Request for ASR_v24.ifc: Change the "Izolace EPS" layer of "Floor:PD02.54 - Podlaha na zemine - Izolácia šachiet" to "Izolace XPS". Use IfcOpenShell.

First a look at what the model holds.

```python
import ifcopenshell
import ifcopenshell.util.element

model = ifcopenshell.open("ASR_v24.ifc")
print(model.schema)
for layer_set in model.by_type("IfcMaterialLayerSet"):
    if layer_set.LayerSetName == "Floor:PD02.54 - Podlaha na zemine - Izolácia šachiet":
        for layer in layer_set.MaterialLayers:
            print(layer.id(), layer.Material and layer.Material.Name, layer.LayerThickness, sep=" | ")
        print(len(ifcopenshell.util.element.get_elements_by_material(model, layer_set)), "elements and types use it")
print(sorted(m.Name for m in model.by_type("IfcMaterial") if m.Name)[:60])
```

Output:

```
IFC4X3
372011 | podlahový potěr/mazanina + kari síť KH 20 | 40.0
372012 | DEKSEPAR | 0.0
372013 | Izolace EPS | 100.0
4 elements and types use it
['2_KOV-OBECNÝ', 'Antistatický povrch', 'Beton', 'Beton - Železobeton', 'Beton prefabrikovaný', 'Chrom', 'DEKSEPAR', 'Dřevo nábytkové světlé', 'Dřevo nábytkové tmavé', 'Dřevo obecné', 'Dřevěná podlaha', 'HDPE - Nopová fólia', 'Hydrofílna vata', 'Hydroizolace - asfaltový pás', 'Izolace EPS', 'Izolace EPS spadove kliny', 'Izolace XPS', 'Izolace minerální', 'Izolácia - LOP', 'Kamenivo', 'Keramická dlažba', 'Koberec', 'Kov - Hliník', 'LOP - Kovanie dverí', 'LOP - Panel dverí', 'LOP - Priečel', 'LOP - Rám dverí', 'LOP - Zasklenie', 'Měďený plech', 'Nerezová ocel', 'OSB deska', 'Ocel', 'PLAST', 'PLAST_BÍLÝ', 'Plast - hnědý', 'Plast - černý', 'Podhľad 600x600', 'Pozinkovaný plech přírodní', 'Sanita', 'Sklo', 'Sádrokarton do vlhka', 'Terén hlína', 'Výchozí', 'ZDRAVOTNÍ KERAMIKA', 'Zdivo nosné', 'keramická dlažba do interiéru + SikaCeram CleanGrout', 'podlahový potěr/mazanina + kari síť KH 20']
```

```python
import ifcopenshell
import ifcopenshell.api.material

model = ifcopenshell.open("ASR_v24.ifc")

layer_set = next(s for s in model.by_type("IfcMaterialLayerSet") if s.LayerSetName == "Floor:PD02.54 - Podlaha na zemine - Izolácia šachiet")
layer = next(l for l in layer_set.MaterialLayers if l.Material and l.Material.Name == "Izolace EPS")
material = next(m for m in model.by_type("IfcMaterial") if m.Name == "Izolace XPS")

# Point this one layer at the other material; renaming the old one would change it everywhere.
ifcopenshell.api.material.edit_layer(model, layer=layer, attributes={"Name": material.Name}, material=material)

print([l.Material.Name if l.Material else None for l in layer_set.MaterialLayers])

model.write("ASR_v24_edited.ifc")
```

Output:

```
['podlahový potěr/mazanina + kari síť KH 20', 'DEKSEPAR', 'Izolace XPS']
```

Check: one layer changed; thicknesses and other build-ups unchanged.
